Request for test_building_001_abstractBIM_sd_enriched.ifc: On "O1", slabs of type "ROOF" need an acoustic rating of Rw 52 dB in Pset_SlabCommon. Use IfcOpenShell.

First a look at what the model holds.

```python
import ifcopenshell
import ifcopenshell.util.element

model = ifcopenshell.open("test_building_001_abstractBIM_sd_enriched.ifc")
print(model.schema)
storey = next(s for s in model.by_type("IfcBuildingStorey") if s.Name == "O1")
slabs = [e for e in ifcopenshell.util.element.get_decomposition(storey) if e.is_a("IfcSlab")]
seen = {}
for e in slabs:
    element_type = ifcopenshell.util.element.get_type(e)
    key = (element_type.Name if element_type != e and element_type else None, ifcopenshell.util.element.get_pset(e, "Pset_SlabCommon", "AcousticRating"))
    seen[key] = seen.get(key, 0) + 1
for (name, value), count in sorted(seen.items(), key=str):
    print(count, "x", name, "|", value)
```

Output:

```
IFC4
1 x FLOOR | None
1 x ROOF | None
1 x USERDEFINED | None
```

```python
import ifcopenshell
import ifcopenshell.api.pset
import ifcopenshell.util.element

model = ifcopenshell.open("test_building_001_abstractBIM_sd_enriched.ifc")

storey = next(s for s in model.by_type("IfcBuildingStorey") if s.Name == "O1")
slabs = [e for e in ifcopenshell.util.element.get_decomposition(storey) if e.is_a("IfcSlab")]

count = 0
for e in slabs:
    element_type = ifcopenshell.util.element.get_type(e)
    if element_type in (None, e) or element_type.Name != "ROOF":
        continue
    # add_pset returns the element's existing set when there is one.
    pset = ifcopenshell.api.pset.add_pset(model, product=e, name="Pset_SlabCommon")
    ifcopenshell.api.pset.edit_pset(model, pset=pset, properties={"AcousticRating": "Rw 52 dB"})
    count += 1

print(count, "slabs updated")

model.write("test_building_001_abstractBIM_sd_enriched_edited.ifc")
```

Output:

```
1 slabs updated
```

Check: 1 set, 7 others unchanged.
